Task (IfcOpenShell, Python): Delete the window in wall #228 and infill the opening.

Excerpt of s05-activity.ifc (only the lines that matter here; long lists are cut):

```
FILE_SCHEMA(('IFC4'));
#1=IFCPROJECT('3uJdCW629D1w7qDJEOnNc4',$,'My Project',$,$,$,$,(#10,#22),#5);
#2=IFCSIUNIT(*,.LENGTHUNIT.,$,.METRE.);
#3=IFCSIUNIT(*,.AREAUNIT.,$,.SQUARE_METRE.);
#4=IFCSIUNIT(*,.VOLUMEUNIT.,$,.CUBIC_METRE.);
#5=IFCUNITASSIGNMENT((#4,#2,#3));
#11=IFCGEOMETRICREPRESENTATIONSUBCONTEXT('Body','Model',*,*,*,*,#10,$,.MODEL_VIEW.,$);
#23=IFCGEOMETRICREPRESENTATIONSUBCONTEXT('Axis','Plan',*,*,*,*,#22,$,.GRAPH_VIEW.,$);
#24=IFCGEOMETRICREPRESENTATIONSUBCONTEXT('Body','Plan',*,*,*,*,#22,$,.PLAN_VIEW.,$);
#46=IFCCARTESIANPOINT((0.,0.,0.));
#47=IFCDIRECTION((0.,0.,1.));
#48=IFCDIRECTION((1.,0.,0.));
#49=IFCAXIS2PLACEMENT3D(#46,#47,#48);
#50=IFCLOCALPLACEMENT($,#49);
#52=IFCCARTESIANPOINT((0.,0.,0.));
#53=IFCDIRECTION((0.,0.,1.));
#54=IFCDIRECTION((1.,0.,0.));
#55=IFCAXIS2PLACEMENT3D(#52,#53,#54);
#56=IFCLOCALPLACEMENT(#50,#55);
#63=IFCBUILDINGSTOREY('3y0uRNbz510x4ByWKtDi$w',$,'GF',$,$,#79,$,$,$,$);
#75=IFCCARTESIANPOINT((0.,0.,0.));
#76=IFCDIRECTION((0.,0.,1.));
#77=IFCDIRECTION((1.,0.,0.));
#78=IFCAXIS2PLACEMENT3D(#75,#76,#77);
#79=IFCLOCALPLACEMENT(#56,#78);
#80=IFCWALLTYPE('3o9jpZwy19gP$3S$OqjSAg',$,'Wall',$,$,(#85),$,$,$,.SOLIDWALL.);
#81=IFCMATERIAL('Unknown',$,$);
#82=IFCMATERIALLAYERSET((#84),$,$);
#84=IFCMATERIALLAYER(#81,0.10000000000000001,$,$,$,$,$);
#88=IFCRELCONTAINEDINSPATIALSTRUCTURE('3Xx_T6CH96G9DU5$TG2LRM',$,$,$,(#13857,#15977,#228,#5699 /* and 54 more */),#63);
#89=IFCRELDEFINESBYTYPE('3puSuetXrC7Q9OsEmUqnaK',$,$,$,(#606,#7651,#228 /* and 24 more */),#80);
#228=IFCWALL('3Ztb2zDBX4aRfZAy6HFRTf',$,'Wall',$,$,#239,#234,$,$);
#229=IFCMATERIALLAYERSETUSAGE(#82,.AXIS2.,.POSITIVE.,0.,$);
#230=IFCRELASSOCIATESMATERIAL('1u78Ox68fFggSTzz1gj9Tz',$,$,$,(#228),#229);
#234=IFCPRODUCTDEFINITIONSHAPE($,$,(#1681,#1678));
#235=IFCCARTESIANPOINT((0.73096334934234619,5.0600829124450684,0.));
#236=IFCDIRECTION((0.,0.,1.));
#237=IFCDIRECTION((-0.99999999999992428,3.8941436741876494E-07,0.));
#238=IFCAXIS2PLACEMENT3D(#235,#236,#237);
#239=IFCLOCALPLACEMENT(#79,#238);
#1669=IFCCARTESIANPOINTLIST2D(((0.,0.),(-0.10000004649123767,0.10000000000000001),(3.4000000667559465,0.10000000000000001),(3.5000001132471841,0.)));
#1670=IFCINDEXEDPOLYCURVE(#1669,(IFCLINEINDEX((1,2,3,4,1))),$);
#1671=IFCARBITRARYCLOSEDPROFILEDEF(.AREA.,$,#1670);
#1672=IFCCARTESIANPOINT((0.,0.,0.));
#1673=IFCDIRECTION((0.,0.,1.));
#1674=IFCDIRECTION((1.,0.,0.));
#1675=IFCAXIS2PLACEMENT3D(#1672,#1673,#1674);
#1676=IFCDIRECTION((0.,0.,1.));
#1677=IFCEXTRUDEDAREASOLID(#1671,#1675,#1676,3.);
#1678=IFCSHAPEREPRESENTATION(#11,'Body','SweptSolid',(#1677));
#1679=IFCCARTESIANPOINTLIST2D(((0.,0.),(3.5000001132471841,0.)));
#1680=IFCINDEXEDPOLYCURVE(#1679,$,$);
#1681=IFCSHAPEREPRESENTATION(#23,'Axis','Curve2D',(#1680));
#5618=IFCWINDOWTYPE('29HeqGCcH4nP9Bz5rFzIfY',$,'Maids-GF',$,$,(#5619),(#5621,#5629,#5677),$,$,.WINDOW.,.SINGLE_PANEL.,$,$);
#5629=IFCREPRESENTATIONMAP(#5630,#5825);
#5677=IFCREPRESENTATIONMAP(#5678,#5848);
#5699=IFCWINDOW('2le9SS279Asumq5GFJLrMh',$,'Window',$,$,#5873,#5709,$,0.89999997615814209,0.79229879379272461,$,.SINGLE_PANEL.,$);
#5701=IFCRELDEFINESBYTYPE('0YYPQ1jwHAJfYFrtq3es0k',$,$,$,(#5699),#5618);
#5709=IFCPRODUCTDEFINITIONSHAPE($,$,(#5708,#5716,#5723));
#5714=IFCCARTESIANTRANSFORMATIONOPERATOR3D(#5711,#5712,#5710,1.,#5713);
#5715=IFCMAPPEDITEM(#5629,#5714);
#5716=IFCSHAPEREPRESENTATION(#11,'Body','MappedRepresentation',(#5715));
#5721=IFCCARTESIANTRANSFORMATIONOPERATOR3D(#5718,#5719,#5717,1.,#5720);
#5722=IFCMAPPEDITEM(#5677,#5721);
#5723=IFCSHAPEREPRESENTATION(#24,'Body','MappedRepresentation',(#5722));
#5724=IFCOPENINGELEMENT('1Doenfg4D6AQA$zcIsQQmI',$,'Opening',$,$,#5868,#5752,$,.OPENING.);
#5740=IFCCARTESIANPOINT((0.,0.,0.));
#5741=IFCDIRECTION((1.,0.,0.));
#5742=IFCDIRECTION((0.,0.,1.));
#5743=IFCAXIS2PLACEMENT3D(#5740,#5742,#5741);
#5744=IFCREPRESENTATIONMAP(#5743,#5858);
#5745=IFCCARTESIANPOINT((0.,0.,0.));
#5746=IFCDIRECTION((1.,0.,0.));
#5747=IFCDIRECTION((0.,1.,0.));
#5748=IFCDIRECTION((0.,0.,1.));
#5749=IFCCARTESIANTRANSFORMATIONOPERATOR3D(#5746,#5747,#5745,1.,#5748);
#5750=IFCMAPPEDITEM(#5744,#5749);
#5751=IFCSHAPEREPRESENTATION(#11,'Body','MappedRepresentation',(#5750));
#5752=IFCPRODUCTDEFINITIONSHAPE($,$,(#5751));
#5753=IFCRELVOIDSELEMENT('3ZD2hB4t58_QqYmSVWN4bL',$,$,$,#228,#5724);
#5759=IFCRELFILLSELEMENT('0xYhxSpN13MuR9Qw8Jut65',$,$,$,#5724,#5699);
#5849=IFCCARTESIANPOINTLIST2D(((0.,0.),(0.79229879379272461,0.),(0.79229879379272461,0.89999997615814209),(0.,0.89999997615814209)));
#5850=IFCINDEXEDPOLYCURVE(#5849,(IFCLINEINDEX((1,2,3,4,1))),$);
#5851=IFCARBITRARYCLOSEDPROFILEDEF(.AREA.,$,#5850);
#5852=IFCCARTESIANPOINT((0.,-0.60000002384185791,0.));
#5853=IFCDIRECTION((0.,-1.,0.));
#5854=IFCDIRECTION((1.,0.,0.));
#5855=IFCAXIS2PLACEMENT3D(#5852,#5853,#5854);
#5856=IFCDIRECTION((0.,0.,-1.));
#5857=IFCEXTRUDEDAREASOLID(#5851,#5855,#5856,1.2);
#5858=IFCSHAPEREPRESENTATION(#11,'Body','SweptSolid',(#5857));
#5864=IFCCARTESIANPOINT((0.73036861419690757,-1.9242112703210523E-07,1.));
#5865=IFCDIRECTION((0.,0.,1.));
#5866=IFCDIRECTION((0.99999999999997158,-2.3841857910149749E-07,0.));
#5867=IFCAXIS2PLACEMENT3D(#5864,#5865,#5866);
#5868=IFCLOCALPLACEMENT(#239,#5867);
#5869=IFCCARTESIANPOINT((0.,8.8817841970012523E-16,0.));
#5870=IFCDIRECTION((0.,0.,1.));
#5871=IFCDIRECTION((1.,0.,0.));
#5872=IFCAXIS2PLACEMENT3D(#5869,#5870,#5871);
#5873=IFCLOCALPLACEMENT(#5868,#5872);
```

```python
import ifcopenshell
import ifcopenshell.api.feature
import ifcopenshell.api.root
import ifcopenshell.geom
import ifcopenshell.util.shape

model = ifcopenshell.open("s05-activity.ifc")
settings = ifcopenshell.geom.settings()


def volume(element):
    """Net volume in cubic metres, openings subtracted."""
    shape = ifcopenshell.geom.create_shape(settings, element)
    return ifcopenshell.util.shape.get_volume(shape.geometry)


window = model.by_guid("2le9SS279Asumq5GFJLrMh")
opening = window.FillsVoids[0].RelatingOpeningElement
wall = opening.VoidsElements[0].RelatingBuildingElement
before = volume(wall)

ifcopenshell.api.root.remove_product(model, product=window)
ifcopenshell.api.feature.remove_feature(model, feature=opening)

after = volume(wall)

print(f"wall volume {before:.3f} -> {after:.3f} m3")

model.write("s05-activity_updated.ifc")
```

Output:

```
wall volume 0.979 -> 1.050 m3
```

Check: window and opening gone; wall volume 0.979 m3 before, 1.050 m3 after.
